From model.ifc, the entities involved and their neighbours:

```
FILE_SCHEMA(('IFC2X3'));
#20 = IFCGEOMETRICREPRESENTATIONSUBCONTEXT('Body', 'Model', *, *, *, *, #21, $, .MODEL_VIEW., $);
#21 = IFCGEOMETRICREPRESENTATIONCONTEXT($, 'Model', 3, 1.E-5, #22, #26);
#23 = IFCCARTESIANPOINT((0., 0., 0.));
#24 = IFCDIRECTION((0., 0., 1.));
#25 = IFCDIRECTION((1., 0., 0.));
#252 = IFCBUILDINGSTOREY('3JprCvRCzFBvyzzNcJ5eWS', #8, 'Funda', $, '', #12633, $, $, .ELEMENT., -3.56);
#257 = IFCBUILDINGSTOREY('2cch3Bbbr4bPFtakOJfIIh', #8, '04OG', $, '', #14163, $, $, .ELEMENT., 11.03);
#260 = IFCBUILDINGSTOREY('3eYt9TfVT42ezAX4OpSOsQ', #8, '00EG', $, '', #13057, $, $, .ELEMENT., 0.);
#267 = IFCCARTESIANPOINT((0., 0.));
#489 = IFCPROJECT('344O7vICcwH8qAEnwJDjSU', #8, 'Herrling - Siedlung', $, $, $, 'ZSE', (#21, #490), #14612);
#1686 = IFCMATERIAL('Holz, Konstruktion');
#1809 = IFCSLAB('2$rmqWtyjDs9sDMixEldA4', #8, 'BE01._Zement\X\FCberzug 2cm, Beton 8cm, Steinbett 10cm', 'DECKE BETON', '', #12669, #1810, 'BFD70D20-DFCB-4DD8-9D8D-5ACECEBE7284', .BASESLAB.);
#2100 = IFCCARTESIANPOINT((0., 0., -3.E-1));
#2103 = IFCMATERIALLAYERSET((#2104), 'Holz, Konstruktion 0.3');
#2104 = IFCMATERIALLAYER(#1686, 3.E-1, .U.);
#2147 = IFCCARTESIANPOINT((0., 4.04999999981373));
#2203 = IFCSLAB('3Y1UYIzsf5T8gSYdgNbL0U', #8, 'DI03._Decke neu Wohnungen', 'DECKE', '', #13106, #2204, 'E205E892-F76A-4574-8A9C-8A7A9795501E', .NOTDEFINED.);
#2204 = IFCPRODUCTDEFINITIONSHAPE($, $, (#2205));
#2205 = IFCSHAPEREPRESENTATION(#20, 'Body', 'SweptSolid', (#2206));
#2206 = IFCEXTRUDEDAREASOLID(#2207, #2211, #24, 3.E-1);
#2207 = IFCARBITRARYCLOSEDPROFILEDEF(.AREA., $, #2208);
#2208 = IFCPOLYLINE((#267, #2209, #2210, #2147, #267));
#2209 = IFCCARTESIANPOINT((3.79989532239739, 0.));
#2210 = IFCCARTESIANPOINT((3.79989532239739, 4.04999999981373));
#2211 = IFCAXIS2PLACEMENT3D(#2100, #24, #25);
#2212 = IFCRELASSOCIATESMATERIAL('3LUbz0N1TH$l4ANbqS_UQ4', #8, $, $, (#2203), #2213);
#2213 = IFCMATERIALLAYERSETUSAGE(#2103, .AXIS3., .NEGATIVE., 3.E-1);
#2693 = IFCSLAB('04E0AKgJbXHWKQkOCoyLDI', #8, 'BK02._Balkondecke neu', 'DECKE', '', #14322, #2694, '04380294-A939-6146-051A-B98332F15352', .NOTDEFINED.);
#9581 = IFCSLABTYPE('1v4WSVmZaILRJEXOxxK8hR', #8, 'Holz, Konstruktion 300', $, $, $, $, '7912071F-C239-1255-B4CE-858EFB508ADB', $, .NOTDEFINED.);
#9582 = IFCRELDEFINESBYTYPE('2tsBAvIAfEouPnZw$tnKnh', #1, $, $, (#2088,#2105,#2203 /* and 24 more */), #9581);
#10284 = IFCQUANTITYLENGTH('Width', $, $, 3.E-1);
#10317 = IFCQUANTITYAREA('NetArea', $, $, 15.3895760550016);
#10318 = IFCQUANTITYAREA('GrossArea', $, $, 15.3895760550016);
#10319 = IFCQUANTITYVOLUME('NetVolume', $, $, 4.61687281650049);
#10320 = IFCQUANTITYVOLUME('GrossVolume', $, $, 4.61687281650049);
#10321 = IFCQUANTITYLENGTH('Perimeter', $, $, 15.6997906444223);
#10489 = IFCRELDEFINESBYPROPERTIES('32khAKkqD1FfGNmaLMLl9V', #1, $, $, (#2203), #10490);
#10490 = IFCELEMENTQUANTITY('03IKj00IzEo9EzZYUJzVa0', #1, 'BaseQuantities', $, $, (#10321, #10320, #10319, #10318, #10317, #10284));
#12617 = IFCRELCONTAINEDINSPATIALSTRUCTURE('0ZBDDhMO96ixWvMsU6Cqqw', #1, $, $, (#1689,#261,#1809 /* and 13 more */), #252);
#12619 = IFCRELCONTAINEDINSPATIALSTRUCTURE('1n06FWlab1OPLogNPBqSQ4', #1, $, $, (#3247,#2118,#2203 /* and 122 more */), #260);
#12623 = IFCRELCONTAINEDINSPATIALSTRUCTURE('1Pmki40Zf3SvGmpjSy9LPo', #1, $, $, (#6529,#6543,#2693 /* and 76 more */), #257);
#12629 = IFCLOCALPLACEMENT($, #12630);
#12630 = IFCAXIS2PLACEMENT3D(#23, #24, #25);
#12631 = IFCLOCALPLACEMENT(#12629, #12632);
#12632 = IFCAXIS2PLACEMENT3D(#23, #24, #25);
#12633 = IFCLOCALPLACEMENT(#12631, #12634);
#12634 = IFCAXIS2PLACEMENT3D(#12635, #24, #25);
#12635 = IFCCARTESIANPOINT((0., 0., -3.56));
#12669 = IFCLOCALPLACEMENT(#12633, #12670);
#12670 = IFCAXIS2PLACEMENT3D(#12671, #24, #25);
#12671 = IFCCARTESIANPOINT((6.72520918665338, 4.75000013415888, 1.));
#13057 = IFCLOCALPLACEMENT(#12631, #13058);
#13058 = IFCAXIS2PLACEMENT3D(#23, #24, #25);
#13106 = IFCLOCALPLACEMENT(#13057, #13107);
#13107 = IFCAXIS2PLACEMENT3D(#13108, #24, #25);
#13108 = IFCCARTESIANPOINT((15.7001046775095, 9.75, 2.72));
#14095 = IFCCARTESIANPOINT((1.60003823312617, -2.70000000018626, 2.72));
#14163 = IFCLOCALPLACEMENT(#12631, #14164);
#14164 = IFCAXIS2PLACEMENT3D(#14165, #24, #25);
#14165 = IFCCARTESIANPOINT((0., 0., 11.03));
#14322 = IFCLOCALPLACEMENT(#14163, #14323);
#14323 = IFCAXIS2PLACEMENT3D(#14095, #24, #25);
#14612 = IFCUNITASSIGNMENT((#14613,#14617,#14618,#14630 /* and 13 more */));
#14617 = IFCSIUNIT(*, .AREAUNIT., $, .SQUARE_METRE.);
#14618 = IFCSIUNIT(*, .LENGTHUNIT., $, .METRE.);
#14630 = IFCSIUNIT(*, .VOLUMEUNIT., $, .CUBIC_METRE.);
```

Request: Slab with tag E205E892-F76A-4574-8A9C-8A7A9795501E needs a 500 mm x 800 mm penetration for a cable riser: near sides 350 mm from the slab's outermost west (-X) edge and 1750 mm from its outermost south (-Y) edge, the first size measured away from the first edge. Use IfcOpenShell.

```python
import numpy as np
import ifcopenshell
import ifcopenshell.api.feature
import ifcopenshell.api.geometry
import ifcopenshell.api.pset
import ifcopenshell.api.root
import ifcopenshell.geom
import ifcopenshell.util.element
import ifcopenshell.util.placement
import ifcopenshell.util.representation
import ifcopenshell.util.shape
import ifcopenshell.util.unit

model = ifcopenshell.open("model.ifc")
unit_scale = ifcopenshell.util.unit.calculate_unit_scale(model)
area_scale = ifcopenshell.util.unit.calculate_unit_scale(model, "AREAUNIT")
volume_scale = ifcopenshell.util.unit.calculate_unit_scale(model, "VOLUMEUNIT")
settings = ifcopenshell.geom.settings()


def volume(element):
    """Net volume in cubic metres, openings subtracted."""
    shape = ifcopenshell.geom.create_shape(settings, element)
    return ifcopenshell.util.shape.get_volume(shape.geometry)


slab = model.by_guid("3Y1UYIzsf5T8gSYdgNbL0U")
before = volume(slab)

# Extent in the slab's own axes, in metres. The edges named are its -X and -Y sides.
slab_shape = ifcopenshell.geom.create_shape(settings, slab)
vertices = ifcopenshell.util.shape.get_vertices(slab_shape.geometry)
x_min, y_min, bottom = vertices.min(axis=0)
top = vertices[:, 2].max()

opening = ifcopenshell.api.root.create_entity(model, ifc_class="IfcOpeningElement", name="Cable riser opening")
context = ifcopenshell.util.representation.get_context(model, "Model", "Body", "MODEL_VIEW")
width, depth = 0.5, 0.8
outline = [(0.0, 0.0), (width, 0.0), (width, depth), (0.0, depth), (0.0, 0.0)]
# Overshoot both faces by 50 mm so the cut is clean.
shape = ifcopenshell.api.geometry.add_slab_representation(
    model, context=context, depth=top - bottom + 0.1, polyline=outline
)
ifcopenshell.api.geometry.assign_representation(model, product=opening, representation=shape)

matrix = ifcopenshell.util.placement.get_local_placement(slab.ObjectPlacement)
matrix[:, 3] = matrix @ np.append(np.array([x_min + 0.35, y_min + 1.75, bottom - 0.05]) / unit_scale, 1.0)
ifcopenshell.api.geometry.edit_object_placement(model, product=opening, matrix=matrix, is_si=False)
ifcopenshell.api.feature.add_feature(model, feature=opening, element=slab)

after = volume(slab)

# Update the slab's stored quantities.
qto = model.by_id(ifcopenshell.util.element.get_pset(slab, "BaseQuantities", should_inherit=False)["id"])
ifcopenshell.api.pset.edit_qto(model, qto=qto, properties={
    "NetVolume": after / volume_scale,
    "NetArea": after / (top - bottom) / area_scale,
})

print(f"slab volume {before:.3f} -> {after:.3f} m3")

model.write("model_updated.ifc")
```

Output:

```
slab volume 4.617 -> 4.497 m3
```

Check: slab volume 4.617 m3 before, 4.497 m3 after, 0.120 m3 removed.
